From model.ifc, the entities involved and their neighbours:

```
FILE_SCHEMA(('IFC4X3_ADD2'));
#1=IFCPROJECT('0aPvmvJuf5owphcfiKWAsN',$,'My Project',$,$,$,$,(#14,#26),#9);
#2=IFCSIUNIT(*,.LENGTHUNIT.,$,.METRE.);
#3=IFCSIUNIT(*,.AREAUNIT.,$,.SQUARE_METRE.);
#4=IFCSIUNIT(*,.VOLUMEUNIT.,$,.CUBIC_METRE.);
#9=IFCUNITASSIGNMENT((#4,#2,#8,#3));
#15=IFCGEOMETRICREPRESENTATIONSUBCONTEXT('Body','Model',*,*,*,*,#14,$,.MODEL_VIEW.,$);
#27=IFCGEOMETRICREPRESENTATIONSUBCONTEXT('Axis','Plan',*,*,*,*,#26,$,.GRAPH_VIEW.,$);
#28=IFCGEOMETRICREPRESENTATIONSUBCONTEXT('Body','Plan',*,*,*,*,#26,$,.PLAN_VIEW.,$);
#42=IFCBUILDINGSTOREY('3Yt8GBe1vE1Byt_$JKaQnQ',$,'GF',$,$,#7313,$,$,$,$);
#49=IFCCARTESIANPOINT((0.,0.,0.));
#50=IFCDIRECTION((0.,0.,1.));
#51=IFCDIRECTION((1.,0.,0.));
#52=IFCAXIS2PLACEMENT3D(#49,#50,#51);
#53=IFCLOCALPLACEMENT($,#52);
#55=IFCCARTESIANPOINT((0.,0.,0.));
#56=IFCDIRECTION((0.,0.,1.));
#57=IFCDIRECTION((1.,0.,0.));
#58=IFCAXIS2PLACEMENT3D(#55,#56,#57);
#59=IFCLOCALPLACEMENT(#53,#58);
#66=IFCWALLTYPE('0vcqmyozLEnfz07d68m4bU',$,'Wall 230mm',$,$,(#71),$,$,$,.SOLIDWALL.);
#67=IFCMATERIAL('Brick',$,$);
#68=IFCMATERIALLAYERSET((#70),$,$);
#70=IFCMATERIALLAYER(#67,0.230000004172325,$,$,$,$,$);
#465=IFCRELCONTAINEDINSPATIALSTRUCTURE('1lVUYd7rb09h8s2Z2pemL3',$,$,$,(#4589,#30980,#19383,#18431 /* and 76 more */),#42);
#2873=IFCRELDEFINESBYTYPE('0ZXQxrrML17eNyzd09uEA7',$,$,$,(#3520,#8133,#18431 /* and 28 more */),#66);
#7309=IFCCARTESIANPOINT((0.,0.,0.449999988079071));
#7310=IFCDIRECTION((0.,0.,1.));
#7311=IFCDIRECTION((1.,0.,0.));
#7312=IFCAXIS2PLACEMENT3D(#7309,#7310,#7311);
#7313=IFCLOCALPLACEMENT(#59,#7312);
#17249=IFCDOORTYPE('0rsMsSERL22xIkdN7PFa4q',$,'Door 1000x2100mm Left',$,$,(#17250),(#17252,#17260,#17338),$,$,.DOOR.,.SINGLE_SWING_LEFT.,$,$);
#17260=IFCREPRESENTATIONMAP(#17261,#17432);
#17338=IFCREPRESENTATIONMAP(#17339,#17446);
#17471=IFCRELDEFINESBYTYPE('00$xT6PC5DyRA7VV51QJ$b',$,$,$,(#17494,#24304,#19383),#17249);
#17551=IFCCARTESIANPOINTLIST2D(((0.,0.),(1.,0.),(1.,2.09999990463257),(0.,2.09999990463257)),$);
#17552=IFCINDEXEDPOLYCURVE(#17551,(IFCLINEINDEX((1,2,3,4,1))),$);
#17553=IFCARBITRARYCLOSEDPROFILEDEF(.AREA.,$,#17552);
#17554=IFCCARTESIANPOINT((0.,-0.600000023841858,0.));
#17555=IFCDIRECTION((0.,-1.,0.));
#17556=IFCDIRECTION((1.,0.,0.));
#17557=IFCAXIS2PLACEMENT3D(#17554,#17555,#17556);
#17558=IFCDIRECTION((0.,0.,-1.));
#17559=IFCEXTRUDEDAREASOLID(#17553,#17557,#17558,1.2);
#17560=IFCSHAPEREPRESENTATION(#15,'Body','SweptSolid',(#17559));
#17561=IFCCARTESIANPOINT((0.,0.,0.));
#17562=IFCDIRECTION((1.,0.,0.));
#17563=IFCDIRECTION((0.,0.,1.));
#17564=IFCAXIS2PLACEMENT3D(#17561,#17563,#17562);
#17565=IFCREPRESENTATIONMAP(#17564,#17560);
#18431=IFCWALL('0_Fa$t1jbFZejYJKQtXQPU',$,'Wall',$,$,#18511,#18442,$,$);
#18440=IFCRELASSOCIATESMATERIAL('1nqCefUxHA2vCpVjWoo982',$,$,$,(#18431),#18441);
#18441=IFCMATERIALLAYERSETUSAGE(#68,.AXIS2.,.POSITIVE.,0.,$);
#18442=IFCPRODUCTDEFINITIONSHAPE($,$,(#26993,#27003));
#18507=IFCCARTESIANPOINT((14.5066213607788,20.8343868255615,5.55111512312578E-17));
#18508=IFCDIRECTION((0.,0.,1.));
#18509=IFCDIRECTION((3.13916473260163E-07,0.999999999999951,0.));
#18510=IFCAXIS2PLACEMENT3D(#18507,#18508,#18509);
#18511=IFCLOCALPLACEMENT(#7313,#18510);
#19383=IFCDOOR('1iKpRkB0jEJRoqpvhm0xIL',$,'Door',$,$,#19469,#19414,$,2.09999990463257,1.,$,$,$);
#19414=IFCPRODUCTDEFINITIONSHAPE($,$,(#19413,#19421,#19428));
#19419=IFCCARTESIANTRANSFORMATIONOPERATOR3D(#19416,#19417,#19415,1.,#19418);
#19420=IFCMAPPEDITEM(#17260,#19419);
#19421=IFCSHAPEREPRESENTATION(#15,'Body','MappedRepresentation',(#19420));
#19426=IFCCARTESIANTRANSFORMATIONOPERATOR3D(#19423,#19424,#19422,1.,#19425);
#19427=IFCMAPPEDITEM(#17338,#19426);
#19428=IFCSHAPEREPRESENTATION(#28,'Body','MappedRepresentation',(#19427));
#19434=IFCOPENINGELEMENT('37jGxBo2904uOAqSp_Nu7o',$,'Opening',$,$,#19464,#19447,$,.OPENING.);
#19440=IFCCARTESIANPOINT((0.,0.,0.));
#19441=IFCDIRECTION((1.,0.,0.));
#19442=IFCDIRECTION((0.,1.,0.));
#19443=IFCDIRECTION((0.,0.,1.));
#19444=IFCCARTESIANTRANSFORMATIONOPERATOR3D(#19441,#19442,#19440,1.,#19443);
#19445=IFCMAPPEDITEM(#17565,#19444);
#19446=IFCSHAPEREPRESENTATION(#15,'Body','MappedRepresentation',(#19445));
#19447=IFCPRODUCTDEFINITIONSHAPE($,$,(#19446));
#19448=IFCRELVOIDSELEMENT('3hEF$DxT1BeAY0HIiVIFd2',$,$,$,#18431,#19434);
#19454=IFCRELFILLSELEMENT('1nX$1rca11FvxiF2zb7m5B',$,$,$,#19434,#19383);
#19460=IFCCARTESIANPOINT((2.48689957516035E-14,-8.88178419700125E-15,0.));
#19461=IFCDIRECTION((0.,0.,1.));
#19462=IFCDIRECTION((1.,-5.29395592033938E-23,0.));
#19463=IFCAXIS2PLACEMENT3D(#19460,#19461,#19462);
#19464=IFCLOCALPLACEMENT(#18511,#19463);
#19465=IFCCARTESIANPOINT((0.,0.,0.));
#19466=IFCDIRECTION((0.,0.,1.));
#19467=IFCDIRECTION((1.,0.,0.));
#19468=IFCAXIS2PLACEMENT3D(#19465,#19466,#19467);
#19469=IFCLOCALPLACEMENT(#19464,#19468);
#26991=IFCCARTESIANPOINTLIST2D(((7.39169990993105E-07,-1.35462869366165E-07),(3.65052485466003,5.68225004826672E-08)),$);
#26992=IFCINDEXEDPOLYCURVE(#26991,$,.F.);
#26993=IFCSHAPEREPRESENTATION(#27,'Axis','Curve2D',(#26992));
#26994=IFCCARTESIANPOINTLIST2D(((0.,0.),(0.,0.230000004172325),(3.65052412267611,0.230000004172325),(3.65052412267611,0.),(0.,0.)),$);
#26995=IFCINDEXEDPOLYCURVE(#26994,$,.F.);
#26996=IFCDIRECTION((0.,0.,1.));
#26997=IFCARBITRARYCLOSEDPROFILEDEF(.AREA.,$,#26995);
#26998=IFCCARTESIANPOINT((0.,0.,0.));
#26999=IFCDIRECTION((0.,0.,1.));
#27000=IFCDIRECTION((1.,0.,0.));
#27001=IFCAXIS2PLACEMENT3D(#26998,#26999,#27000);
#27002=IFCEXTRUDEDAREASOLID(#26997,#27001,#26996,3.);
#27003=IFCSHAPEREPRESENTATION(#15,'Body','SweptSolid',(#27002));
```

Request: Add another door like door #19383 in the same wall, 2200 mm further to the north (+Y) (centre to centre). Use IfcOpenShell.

```python
import ifcopenshell
import ifcopenshell.api.feature
import ifcopenshell.api.geometry
import ifcopenshell.api.root
import ifcopenshell.geom
import ifcopenshell.util.element
import ifcopenshell.util.placement
import ifcopenshell.util.shape
import ifcopenshell.util.unit

model = ifcopenshell.open("model.ifc")
unit_scale = ifcopenshell.util.unit.calculate_unit_scale(model)
settings = ifcopenshell.geom.settings()


def volume(element):
    """Net volume in cubic metres, openings subtracted."""
    shape = ifcopenshell.geom.create_shape(settings, element)
    return ifcopenshell.util.shape.get_volume(shape.geometry)


door = model.by_id(19383)
opening = door.FillsVoids[0].RelatingOpeningElement
wall = opening.VoidsElements[0].RelatingBuildingElement
before = volume(wall)
shift = ifcopenshell.util.placement.get_local_placement(wall.ObjectPlacement)[:3, 0] * 2.2 / unit_scale

# copy_class copies the void relationship, type, container and properties, but no geometry.
new_opening = ifcopenshell.api.root.copy_class(model, product=opening)
new_opening.Representation = ifcopenshell.util.element.copy_deep(
    model, opening.Representation, exclude=["IfcGeometricRepresentationContext", "IfcRepresentationMap"]
)
new_door = ifcopenshell.api.root.copy_class(model, product=door)
new_door.Representation = ifcopenshell.util.element.copy_deep(
    model, door.Representation, exclude=["IfcGeometricRepresentationContext", "IfcRepresentationMap"]
)
ifcopenshell.api.feature.add_filling(model, opening=new_opening, element=new_door)

for old, new in ((opening, new_opening), (door, new_door)):
    matrix = ifcopenshell.util.placement.get_local_placement(old.ObjectPlacement)
    matrix[:3, 3] += shift
    ifcopenshell.api.geometry.edit_object_placement(model, product=new, matrix=matrix, is_si=False)

after = volume(wall)

print(f"wall volume {before:.3f} -> {after:.3f} m3")

model.write("model-out.ifc")
```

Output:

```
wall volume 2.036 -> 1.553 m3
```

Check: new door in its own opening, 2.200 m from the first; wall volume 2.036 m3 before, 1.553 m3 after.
